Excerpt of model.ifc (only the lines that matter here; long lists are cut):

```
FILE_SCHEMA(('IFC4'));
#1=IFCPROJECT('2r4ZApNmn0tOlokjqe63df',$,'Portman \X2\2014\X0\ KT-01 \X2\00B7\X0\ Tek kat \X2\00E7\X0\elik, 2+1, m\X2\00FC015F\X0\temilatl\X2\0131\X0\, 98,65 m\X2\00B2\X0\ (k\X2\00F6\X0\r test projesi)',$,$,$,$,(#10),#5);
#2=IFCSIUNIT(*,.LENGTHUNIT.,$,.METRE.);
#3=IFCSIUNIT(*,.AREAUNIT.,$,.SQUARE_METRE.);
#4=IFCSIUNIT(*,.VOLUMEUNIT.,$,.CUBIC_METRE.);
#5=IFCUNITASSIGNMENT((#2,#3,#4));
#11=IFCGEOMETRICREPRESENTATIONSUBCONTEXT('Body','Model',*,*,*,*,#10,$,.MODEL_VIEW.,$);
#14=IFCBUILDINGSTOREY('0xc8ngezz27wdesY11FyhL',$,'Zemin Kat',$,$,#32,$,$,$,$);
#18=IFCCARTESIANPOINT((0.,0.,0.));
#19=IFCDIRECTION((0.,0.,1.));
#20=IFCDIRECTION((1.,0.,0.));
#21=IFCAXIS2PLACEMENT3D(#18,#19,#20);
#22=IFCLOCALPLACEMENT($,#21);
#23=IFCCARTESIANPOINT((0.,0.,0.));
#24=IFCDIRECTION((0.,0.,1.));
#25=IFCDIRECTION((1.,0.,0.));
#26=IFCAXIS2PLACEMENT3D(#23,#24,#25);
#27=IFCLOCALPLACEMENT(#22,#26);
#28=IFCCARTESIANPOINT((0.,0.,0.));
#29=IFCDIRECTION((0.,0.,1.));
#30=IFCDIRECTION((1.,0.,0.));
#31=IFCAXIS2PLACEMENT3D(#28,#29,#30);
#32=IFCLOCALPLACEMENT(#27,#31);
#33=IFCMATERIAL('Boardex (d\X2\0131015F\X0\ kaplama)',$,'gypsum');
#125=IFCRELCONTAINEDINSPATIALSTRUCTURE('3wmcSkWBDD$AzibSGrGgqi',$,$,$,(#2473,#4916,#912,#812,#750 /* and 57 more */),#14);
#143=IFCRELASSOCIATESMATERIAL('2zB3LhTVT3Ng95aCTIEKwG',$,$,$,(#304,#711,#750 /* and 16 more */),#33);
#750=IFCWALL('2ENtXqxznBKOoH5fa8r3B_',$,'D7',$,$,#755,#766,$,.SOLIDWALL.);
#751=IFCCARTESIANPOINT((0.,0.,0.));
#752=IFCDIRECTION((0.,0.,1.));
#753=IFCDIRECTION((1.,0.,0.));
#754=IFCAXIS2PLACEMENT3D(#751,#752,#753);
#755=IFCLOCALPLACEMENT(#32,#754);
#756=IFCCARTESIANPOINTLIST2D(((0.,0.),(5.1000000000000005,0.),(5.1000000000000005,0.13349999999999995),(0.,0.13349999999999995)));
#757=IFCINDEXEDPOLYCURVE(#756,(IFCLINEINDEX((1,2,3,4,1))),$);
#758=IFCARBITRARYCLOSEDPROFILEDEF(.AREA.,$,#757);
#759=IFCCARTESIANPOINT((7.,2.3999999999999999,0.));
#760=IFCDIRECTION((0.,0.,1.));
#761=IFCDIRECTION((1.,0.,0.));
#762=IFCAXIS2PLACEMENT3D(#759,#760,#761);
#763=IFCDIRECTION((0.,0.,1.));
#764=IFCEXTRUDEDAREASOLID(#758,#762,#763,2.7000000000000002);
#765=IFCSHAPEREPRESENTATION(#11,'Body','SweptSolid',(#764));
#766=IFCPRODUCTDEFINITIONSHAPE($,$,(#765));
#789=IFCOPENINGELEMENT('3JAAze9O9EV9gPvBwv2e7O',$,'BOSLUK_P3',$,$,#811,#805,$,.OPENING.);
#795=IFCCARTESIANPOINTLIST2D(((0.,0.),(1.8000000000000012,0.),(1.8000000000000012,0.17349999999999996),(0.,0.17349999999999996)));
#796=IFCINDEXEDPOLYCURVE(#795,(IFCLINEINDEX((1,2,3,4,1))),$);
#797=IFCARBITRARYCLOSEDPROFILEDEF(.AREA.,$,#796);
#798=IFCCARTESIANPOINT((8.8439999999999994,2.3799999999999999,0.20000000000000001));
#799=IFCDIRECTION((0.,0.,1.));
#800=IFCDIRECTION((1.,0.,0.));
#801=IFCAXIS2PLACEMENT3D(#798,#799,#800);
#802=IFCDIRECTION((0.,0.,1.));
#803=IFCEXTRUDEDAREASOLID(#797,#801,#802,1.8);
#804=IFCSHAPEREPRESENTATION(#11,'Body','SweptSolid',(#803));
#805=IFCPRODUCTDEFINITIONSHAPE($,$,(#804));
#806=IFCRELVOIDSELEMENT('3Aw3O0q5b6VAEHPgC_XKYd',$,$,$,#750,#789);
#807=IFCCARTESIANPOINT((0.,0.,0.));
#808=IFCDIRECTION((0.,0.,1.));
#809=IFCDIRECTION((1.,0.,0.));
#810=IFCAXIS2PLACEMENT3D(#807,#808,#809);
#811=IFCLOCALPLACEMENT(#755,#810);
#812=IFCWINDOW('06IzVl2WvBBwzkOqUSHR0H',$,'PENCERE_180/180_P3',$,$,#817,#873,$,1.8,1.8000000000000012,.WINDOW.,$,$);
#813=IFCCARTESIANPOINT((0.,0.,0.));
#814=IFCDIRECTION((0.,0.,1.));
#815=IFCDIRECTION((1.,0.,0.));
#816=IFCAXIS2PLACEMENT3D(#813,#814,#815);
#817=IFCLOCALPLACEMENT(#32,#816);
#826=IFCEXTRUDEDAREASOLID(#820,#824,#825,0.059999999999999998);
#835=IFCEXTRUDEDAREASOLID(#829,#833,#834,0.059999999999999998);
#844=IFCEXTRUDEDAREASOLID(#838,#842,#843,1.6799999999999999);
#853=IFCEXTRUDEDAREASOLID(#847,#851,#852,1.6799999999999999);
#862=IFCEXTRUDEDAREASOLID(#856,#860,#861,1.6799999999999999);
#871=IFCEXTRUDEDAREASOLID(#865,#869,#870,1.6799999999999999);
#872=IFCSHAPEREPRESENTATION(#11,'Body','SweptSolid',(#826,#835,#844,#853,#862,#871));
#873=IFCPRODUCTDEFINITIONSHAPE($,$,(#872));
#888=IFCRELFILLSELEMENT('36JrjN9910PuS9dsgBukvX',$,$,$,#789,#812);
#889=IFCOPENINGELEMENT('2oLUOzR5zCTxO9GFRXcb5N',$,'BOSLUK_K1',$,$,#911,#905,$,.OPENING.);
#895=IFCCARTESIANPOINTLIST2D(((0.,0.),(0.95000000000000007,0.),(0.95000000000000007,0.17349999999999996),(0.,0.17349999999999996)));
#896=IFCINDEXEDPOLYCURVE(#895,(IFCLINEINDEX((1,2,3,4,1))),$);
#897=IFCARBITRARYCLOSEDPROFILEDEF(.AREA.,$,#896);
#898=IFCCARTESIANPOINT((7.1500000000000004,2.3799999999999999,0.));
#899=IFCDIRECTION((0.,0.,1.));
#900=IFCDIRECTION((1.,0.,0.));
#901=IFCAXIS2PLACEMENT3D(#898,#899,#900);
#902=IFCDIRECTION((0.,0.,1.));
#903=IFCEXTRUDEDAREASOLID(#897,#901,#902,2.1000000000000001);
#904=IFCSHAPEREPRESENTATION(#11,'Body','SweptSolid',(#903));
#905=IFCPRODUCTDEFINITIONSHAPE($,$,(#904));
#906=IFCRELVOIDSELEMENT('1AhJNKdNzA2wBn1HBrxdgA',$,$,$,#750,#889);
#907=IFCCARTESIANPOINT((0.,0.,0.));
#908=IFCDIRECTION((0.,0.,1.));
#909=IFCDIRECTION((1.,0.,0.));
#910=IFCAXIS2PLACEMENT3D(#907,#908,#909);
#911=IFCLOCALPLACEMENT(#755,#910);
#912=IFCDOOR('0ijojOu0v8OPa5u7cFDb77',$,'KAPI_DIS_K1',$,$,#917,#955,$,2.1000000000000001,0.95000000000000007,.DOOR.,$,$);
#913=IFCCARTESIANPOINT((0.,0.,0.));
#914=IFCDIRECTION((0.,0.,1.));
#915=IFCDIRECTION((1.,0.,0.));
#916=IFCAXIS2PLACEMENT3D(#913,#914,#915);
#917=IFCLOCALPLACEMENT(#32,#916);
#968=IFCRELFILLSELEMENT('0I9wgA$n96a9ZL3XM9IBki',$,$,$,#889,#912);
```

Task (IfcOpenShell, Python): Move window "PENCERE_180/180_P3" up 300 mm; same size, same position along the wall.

```python
import numpy as np
import ifcopenshell
import ifcopenshell.api.geometry
import ifcopenshell.util.placement
import ifcopenshell.util.unit

model = ifcopenshell.open("model.ifc")
unit_scale = ifcopenshell.util.unit.calculate_unit_scale(model)

window = model.by_guid("06IzVl2WvBBwzkOqUSHR0H")
opening = window.FillsVoids[0].RelatingOpeningElement
dz = 0.3 / unit_scale

shift = np.array([0.0, 0.0, dz])
# The window is not placed relative to its opening, so move both.
for product in (opening, window):
    matrix = ifcopenshell.util.placement.get_local_placement(product.ObjectPlacement)
    matrix[:3, 3] += shift
    ifcopenshell.api.geometry.edit_object_placement(model, product=product, matrix=matrix, is_si=False)

print(f"moved by {dz * unit_scale:+.3f} m")

model.write("model_v2.ifc")
```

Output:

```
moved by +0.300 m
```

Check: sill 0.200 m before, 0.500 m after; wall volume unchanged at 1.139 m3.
